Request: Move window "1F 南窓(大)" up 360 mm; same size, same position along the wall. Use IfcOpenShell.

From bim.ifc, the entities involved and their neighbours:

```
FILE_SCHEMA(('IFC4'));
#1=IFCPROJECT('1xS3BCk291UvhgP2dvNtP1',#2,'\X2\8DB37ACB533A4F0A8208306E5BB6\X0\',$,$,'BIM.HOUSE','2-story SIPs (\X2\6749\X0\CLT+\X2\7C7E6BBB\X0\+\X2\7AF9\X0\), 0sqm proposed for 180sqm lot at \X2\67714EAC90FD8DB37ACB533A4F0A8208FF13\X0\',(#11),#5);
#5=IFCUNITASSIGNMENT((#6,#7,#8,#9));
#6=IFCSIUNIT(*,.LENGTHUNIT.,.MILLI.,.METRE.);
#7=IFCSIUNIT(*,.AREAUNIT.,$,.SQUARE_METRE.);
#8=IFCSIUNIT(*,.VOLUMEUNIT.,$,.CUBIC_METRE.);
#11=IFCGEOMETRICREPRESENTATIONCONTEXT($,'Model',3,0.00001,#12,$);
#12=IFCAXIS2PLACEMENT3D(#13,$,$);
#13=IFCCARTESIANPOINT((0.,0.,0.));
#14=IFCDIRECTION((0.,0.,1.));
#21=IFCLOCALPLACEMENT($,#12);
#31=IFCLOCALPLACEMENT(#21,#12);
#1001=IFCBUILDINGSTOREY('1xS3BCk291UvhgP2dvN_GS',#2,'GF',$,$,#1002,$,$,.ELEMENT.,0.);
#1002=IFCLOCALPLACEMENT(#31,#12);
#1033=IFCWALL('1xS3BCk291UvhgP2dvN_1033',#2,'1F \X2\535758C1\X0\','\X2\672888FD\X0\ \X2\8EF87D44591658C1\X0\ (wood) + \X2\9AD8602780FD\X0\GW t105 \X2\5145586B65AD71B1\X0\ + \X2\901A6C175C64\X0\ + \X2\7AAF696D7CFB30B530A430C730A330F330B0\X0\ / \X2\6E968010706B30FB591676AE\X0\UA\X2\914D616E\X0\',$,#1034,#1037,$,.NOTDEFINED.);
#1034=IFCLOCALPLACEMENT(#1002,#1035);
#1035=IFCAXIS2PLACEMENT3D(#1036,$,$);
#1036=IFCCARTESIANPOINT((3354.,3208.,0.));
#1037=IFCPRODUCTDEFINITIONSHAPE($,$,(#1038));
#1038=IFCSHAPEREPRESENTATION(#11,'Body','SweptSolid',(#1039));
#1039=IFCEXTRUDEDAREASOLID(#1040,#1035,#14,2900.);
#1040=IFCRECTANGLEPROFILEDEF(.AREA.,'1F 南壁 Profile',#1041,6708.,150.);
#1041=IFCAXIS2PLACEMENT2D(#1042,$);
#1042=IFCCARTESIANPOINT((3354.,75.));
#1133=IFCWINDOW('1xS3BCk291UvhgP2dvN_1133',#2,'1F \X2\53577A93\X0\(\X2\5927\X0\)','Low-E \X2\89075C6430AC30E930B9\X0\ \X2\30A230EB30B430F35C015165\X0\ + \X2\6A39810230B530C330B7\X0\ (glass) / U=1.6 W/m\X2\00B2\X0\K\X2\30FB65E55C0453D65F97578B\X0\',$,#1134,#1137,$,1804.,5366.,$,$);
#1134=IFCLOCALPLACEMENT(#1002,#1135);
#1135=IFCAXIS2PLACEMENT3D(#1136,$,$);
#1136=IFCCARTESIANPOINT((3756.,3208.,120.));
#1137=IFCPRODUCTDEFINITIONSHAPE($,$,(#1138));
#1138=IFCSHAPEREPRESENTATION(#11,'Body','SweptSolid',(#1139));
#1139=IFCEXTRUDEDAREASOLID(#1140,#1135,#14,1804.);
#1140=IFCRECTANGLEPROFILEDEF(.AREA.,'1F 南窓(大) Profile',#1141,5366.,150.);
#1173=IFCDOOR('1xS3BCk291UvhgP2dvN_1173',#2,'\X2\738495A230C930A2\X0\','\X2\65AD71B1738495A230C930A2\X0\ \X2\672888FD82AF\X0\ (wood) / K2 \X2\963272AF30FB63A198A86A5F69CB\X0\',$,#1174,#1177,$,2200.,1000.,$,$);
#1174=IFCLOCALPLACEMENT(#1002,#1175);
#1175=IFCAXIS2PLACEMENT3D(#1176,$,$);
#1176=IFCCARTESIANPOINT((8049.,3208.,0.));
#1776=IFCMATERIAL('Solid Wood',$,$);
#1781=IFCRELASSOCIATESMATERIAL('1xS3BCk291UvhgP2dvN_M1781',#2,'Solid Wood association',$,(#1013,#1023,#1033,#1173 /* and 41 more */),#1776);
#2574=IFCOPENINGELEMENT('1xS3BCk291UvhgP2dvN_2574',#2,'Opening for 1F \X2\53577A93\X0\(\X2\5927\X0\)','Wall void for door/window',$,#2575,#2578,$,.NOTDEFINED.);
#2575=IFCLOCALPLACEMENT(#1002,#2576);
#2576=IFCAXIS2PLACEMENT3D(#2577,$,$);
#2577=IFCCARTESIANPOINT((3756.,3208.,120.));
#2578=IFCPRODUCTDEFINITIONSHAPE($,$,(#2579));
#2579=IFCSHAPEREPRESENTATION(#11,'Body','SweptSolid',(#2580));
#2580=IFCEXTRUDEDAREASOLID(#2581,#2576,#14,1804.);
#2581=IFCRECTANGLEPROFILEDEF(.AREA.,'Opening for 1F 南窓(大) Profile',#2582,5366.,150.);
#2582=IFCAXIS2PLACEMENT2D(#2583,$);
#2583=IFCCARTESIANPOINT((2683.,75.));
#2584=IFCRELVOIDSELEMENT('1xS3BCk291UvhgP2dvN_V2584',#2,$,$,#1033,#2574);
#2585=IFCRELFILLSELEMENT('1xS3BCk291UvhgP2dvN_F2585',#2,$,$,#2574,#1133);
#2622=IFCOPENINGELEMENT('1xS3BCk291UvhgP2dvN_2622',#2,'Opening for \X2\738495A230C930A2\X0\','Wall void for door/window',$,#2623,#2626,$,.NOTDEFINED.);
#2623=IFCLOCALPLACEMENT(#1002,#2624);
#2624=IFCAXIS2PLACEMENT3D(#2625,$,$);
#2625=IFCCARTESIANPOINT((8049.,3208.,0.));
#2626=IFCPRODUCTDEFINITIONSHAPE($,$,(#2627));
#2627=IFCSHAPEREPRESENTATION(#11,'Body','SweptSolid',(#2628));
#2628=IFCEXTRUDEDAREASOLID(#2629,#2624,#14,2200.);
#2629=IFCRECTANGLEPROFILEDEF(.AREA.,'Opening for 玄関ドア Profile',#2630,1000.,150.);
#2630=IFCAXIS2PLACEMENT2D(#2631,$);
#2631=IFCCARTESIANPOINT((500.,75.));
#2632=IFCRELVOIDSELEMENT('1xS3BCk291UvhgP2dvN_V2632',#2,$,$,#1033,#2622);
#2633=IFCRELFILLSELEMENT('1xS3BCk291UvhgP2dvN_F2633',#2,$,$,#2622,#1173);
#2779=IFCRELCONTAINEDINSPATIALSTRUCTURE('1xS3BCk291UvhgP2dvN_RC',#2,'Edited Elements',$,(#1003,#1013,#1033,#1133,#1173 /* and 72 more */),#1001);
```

```python
import numpy as np
import ifcopenshell
import ifcopenshell.api.geometry
import ifcopenshell.util.placement
import ifcopenshell.util.unit

model = ifcopenshell.open("bim.ifc")
unit_scale = ifcopenshell.util.unit.calculate_unit_scale(model)

window = model.by_guid("1xS3BCk291UvhgP2dvN_1133")
opening = window.FillsVoids[0].RelatingOpeningElement
dz = 0.36 / unit_scale

shift = np.array([0.0, 0.0, dz])
# The window is not placed relative to its opening, so move both.
for product in (opening, window):
    matrix = ifcopenshell.util.placement.get_local_placement(product.ObjectPlacement)
    matrix[:3, 3] += shift
    ifcopenshell.api.geometry.edit_object_placement(model, product=product, matrix=matrix, is_si=False)

print(f"moved by {dz * unit_scale:+.3f} m")

model.write("bim_v2.ifc")
```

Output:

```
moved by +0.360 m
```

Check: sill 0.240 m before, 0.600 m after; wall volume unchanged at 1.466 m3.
